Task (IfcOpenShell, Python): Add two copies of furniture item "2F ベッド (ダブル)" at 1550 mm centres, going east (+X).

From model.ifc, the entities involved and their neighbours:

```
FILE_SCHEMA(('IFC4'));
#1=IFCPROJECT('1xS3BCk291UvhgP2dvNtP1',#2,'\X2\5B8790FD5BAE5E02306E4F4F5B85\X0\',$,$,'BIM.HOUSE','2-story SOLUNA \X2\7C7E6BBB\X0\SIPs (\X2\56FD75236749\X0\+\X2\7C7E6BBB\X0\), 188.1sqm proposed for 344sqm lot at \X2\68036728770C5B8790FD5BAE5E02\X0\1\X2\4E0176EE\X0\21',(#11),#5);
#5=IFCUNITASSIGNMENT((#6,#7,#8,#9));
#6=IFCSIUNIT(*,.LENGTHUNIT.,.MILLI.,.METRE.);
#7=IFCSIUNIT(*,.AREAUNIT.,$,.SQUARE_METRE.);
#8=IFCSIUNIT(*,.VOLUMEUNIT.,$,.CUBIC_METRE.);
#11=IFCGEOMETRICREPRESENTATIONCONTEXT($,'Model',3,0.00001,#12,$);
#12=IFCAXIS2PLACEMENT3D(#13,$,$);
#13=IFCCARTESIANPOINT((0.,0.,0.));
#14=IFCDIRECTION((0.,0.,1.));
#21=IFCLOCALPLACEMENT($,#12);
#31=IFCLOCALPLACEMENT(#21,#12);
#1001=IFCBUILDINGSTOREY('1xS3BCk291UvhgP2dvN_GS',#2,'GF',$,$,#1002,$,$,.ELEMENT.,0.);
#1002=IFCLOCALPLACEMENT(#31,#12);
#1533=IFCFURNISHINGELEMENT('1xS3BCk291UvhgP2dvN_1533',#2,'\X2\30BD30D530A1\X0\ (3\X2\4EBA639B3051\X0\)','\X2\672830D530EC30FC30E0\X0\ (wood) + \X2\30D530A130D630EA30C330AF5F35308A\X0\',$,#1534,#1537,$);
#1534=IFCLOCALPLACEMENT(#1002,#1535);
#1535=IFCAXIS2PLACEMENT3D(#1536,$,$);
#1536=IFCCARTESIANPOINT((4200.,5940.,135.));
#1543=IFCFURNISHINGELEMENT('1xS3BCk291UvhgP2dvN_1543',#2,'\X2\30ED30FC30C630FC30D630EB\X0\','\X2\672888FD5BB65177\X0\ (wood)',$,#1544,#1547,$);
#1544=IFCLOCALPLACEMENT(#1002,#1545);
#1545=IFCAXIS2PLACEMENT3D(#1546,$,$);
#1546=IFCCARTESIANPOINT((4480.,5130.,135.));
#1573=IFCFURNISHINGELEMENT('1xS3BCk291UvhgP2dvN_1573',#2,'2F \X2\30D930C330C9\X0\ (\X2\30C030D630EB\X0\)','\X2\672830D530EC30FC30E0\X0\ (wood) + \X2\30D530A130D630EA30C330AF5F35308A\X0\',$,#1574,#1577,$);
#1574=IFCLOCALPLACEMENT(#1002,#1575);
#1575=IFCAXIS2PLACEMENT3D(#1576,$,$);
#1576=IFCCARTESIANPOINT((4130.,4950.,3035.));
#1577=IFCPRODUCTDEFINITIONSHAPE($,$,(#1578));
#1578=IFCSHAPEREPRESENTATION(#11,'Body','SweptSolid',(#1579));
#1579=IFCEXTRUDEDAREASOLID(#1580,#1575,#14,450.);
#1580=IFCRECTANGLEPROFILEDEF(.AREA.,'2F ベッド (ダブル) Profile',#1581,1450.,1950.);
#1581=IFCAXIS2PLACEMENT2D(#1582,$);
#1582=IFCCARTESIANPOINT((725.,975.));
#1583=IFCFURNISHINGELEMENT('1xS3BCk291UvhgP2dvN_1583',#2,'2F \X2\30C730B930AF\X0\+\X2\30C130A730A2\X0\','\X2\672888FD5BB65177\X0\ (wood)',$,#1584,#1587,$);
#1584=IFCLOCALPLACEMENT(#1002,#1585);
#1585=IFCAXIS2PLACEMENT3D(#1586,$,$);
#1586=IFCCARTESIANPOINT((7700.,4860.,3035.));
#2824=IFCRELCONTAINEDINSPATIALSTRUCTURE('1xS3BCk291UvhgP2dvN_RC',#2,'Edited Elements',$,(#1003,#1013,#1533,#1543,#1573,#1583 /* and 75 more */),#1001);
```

```python
import numpy as np
import ifcopenshell
import ifcopenshell.api.geometry
import ifcopenshell.api.root
import ifcopenshell.util.element
import ifcopenshell.util.placement
import ifcopenshell.util.unit

model = ifcopenshell.open("model.ifc")
unit_scale = ifcopenshell.util.unit.calculate_unit_scale(model)


def reuse_history(source, copy):
    """copy_class also copies each property set's owner history, people and application; keep the originals."""
    for rel in copy.IsDefinedBy:
        if rel.is_a("IfcRelDefinesByProperties") and (history := rel.RelatingPropertyDefinition.OwnerHistory):
            rel.RelatingPropertyDefinition.OwnerHistory = source.OwnerHistory
            ifcopenshell.util.element.remove_deep2(model, history)


source = model.by_guid("1xS3BCk291UvhgP2dvN_1573")
base = ifcopenshell.util.placement.get_local_placement(source.ObjectPlacement)
step = np.array([1.0, 0.0, 0.0]) * 1.55 / unit_scale

for i in range(1, 3):
    copy = ifcopenshell.api.root.copy_class(model, product=source)
    copy.Representation = ifcopenshell.util.element.copy_deep(
        model, source.Representation, exclude=["IfcGeometricRepresentationContext", "IfcRepresentationMap"]
    )
    reuse_history(source, copy)
    matrix = base.copy()
    matrix[:3, 3] += i * step
    print("added at", matrix[:3, 3].round(3) + 0.0)
    ifcopenshell.api.geometry.edit_object_placement(model, product=copy, matrix=matrix, is_si=False)

model.write("model_rev.ifc")
```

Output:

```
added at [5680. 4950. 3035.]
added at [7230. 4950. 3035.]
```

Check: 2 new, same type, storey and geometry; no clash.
